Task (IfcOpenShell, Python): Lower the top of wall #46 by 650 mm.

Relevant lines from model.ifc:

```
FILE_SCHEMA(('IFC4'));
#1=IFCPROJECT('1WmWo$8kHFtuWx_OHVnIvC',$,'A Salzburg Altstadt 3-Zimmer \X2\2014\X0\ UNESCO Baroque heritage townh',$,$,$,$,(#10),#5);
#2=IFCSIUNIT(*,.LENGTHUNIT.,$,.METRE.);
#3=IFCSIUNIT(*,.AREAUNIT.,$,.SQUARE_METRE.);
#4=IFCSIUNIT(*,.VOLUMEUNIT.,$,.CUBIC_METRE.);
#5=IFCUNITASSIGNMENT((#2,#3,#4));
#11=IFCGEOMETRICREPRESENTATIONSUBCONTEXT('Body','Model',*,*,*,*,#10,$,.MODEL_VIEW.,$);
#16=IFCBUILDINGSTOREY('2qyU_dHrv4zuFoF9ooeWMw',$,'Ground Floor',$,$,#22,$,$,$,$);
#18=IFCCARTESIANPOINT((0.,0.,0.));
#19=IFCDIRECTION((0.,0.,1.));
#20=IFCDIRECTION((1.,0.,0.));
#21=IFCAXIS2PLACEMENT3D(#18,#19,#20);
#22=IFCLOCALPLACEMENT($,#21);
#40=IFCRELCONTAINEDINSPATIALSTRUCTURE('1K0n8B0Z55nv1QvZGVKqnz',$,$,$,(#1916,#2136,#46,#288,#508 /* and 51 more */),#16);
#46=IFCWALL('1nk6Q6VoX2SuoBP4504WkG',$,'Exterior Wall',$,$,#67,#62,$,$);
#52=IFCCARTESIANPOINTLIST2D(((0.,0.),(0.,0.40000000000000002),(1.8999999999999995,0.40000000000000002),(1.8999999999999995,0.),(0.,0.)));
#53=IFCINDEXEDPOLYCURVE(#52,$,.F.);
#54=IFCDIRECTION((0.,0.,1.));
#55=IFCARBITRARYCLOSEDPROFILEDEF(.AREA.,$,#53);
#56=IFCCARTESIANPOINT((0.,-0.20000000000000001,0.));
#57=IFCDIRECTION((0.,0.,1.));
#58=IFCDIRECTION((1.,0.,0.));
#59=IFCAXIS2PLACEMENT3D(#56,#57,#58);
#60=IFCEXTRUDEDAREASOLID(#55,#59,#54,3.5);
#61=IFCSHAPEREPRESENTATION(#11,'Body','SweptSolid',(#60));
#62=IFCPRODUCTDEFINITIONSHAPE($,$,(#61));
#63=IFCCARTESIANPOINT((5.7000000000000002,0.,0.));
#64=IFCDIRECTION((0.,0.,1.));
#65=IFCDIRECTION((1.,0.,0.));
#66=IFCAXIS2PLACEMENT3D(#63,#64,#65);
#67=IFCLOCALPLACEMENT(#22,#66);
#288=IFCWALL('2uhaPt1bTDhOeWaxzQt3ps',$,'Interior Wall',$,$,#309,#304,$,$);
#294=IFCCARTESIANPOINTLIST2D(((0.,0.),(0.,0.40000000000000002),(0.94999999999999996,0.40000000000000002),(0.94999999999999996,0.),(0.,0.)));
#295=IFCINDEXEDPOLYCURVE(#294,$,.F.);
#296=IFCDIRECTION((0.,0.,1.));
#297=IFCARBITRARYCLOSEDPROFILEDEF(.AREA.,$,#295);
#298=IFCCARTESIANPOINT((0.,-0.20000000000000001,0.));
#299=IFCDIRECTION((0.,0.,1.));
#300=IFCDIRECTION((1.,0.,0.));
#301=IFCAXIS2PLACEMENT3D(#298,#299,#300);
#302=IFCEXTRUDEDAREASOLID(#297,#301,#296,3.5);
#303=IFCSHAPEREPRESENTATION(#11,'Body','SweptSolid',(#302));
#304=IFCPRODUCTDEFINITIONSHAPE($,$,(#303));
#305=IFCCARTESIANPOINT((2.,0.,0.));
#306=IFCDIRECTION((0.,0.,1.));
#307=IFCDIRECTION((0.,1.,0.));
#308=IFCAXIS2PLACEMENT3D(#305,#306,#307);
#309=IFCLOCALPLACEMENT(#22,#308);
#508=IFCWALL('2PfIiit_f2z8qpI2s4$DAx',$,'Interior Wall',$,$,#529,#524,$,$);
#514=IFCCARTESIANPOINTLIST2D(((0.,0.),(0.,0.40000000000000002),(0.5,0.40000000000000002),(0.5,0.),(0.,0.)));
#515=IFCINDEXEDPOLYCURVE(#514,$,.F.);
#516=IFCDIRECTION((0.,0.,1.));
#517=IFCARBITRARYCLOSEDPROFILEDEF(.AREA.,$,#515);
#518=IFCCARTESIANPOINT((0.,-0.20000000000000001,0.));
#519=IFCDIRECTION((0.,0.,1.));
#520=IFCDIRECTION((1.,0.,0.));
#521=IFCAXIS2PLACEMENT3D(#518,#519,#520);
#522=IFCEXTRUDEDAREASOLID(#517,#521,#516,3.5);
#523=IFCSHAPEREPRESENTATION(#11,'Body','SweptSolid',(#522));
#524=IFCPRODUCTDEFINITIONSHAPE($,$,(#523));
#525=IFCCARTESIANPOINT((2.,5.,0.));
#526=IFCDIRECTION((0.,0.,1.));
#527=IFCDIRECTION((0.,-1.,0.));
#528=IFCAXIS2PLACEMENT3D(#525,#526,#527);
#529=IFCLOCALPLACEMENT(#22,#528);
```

```python
import ifcopenshell
import ifcopenshell.geom
import ifcopenshell.util.representation
import ifcopenshell.util.shape

model = ifcopenshell.open("model.ifc")
settings = ifcopenshell.geom.settings()


def volume(element):
    """Net volume in cubic metres, openings subtracted."""
    shape = ifcopenshell.geom.create_shape(settings, element)
    return ifcopenshell.util.shape.get_volume(shape.geometry)


wall = model.by_guid("1nk6Q6VoX2SuoBP4504WkG")
before = volume(wall)

body = ifcopenshell.util.representation.get_representation(wall, "Model", "Body")
solid = body.Items[0]
old_height = solid.Depth
solid.Depth -= 0.65
after = volume(wall)

print(f"height {old_height:g} -> {solid.Depth:g}, volume {before:.3f} -> {after:.3f} m3")

model.write("model_updated.ifc")
```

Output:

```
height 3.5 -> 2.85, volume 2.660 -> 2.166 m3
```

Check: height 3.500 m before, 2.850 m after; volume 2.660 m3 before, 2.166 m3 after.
